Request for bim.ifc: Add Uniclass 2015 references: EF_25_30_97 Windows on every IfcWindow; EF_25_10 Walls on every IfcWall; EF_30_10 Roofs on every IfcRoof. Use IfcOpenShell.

First a look at what the model holds.

```python
import ifcopenshell

model = ifcopenshell.open("bim.ifc")
print(model.schema)
print("classifications:", [c.Name for c in model.by_type("IfcClassification")])
for ifc_class in ("IfcDoor", "IfcRoof", "IfcStair", "IfcWall", "IfcWindow"):
    print(ifc_class, len(model.by_type(ifc_class)))
```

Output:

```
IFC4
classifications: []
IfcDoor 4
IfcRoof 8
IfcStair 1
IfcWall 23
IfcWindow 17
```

```python
import ifcopenshell
import ifcopenshell.api.classification

model = ifcopenshell.open("bim.ifc")

system = ifcopenshell.api.classification.add_classification(model, classification="Uniclass 2015")

codes = {
    "IfcWindow": ("EF_25_30_97", "Windows"),
    "IfcWall": ("EF_25_10", "Walls"),
    "IfcRoof": ("EF_30_10", "Roofs"),
}
for ifc_class, (code, name) in codes.items():
    products = model.by_type(ifc_class)
    ifcopenshell.api.classification.add_reference(
        model, products=products, classification=system, identification=code, name=name
    )
    print(code, len(products))

model.write("bim-out.ifc")
```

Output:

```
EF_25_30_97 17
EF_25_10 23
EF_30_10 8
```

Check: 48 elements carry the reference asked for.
